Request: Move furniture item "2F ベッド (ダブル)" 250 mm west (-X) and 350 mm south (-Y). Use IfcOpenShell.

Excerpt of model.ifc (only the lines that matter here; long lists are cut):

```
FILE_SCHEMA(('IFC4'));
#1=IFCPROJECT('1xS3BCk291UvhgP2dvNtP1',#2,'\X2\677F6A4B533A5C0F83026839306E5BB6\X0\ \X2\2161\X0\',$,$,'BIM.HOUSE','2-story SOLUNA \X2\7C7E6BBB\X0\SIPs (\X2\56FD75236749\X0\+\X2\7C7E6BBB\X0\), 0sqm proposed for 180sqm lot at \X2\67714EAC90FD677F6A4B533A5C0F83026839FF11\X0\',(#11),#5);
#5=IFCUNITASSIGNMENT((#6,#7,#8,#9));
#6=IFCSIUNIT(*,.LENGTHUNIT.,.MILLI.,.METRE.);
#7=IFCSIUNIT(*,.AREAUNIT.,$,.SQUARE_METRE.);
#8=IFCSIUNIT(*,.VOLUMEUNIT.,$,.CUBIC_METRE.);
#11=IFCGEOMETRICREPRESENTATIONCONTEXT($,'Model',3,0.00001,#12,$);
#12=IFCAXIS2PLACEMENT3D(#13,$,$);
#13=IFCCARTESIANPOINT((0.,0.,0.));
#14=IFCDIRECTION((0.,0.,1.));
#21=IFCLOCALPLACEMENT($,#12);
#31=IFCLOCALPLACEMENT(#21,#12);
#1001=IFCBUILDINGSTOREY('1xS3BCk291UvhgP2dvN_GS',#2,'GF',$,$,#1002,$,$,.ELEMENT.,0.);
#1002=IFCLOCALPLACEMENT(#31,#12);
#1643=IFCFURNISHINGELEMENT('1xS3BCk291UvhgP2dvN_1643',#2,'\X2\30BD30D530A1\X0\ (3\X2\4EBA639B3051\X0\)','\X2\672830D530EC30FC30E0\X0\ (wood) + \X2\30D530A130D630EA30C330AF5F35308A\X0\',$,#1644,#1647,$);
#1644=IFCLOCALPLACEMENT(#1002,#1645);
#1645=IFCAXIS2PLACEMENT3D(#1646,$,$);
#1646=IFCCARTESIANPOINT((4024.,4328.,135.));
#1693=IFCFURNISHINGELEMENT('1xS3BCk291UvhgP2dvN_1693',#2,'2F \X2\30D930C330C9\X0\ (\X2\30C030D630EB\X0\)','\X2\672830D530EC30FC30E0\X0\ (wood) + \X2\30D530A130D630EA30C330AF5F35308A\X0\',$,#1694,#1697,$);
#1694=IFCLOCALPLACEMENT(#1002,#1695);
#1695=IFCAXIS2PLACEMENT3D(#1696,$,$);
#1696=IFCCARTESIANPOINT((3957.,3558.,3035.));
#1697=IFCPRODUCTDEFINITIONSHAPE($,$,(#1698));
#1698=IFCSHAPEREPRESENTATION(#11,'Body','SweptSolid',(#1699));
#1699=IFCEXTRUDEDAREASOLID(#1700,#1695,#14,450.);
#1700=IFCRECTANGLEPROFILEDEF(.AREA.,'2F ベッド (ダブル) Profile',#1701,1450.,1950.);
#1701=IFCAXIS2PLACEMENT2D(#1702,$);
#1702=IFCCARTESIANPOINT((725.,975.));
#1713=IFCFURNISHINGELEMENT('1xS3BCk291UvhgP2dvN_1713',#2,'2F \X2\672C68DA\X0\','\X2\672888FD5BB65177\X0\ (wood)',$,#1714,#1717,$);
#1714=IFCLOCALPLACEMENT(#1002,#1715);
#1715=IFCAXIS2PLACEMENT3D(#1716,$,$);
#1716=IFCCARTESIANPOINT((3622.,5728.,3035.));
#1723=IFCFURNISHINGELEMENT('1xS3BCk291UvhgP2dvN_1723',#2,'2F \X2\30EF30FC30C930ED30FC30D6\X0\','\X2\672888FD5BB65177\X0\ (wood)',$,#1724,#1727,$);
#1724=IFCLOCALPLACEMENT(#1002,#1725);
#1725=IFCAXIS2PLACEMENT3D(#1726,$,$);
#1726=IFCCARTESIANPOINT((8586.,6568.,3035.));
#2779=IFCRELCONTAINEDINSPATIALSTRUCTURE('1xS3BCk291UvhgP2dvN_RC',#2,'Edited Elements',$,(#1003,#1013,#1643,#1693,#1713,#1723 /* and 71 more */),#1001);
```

```python
import ifcopenshell
import ifcopenshell.api.geometry
import ifcopenshell.util.placement
import ifcopenshell.util.unit

model = ifcopenshell.open("model.ifc")
unit_scale = ifcopenshell.util.unit.calculate_unit_scale(model)

item = model.by_id(1693)
matrix = ifcopenshell.util.placement.get_local_placement(item.ObjectPlacement)
matrix[0, 3] -= 0.25 / unit_scale
matrix[1, 3] -= 0.35 / unit_scale
ifcopenshell.api.geometry.edit_object_placement(model, product=item, matrix=matrix, is_si=False)

print(ifcopenshell.util.placement.get_local_placement(item.ObjectPlacement).round(3) + 0.0)

model.write("model_v2.ifc")
```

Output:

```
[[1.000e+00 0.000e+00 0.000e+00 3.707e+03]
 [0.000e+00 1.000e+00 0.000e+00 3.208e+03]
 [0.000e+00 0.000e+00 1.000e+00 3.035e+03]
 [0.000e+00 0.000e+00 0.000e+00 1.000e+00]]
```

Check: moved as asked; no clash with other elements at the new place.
